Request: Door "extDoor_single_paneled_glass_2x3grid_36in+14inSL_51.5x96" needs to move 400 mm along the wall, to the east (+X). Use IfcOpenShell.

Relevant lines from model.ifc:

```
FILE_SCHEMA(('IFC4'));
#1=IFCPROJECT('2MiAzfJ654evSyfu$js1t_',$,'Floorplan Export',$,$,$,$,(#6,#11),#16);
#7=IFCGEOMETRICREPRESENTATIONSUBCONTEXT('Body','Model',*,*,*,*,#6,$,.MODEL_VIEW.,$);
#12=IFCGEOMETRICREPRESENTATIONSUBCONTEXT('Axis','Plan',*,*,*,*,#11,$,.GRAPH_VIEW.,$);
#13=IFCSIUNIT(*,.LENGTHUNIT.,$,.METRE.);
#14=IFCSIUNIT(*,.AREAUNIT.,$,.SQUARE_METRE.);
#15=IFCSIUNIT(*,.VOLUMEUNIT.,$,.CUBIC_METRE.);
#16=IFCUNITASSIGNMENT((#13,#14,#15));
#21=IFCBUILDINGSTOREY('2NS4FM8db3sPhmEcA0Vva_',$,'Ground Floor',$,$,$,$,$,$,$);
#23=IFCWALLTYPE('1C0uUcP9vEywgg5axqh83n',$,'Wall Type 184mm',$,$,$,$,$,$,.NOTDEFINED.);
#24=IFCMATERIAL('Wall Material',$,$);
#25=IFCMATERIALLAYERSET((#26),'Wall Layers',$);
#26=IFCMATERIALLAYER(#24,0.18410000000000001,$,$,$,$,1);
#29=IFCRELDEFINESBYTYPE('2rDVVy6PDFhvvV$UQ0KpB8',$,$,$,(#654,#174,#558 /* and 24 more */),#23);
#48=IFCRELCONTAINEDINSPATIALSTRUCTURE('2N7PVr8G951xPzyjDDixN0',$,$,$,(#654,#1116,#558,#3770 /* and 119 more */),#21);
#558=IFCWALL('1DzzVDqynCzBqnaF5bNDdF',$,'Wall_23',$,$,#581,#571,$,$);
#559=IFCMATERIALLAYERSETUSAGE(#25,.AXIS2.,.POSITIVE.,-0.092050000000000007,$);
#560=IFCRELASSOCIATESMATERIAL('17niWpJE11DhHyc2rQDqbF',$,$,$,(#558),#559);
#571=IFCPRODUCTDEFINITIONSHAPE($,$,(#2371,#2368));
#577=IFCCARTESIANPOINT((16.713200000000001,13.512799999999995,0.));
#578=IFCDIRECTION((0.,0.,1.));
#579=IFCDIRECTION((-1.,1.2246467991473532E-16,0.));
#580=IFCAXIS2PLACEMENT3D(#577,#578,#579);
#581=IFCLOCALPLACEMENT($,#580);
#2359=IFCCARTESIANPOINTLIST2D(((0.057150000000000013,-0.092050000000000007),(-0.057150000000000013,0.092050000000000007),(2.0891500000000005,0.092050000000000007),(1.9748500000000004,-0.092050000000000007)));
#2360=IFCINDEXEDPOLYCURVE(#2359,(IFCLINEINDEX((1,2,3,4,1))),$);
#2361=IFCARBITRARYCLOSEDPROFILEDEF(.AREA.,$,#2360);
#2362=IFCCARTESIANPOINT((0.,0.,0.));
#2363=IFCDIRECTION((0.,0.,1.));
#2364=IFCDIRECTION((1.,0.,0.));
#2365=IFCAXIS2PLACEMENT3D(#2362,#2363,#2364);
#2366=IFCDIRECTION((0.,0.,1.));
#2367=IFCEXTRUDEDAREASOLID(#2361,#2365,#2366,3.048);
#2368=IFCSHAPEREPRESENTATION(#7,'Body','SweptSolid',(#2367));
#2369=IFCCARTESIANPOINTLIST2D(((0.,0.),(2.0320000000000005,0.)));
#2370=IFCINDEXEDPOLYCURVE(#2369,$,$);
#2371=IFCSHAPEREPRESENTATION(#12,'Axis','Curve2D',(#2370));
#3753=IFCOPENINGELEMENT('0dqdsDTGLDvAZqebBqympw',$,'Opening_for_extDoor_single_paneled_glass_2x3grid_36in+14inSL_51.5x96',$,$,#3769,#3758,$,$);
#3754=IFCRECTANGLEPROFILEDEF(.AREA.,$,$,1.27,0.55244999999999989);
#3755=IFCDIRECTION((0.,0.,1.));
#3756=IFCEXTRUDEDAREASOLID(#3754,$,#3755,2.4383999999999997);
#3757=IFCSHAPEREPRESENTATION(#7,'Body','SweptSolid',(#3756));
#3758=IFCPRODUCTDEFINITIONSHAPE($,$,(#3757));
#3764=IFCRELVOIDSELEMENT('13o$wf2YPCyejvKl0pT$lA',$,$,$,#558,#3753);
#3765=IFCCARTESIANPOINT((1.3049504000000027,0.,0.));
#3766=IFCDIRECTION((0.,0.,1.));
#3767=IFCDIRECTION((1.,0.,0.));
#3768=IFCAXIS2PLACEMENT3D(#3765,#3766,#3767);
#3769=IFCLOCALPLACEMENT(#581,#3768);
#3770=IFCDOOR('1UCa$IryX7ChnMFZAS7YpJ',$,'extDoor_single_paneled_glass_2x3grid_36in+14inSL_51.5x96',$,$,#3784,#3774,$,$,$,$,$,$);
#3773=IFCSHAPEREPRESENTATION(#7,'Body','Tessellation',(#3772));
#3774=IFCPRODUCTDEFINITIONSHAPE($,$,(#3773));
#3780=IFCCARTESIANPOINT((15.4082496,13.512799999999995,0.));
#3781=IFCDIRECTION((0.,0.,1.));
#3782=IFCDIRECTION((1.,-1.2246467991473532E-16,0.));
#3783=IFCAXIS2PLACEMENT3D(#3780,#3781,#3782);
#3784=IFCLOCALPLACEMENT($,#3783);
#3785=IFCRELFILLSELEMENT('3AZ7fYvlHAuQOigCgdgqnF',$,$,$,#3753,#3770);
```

```python
import ifcopenshell
import ifcopenshell.api.geometry
import ifcopenshell.util.placement
import ifcopenshell.util.unit

model = ifcopenshell.open("model.ifc")
unit_scale = ifcopenshell.util.unit.calculate_unit_scale(model)

door = model.by_guid("1UCa$IryX7ChnMFZAS7YpJ")
opening = door.FillsVoids[0].RelatingOpeningElement
wall = opening.VoidsElements[0].RelatingBuildingElement

wall_matrix = ifcopenshell.util.placement.get_local_placement(wall.ObjectPlacement)
shift = wall_matrix[:3, 0] * -0.4 / unit_scale
before = ifcopenshell.util.placement.get_local_placement(door.ObjectPlacement)[:3, 3].copy()

# The door is not placed relative to its opening, so move both.
for product in (opening, door):
    matrix = ifcopenshell.util.placement.get_local_placement(product.ObjectPlacement)
    matrix[:3, 3] += shift
    ifcopenshell.api.geometry.edit_object_placement(model, product=product, matrix=matrix, is_si=False)

after = ifcopenshell.util.placement.get_local_placement(door.ObjectPlacement)[:3, 3]
print("door moved by", (after - before).round(3) + 0.0)

model.write("model_rev.ifc")
```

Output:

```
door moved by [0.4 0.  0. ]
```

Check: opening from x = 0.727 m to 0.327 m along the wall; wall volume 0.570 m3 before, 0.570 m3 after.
